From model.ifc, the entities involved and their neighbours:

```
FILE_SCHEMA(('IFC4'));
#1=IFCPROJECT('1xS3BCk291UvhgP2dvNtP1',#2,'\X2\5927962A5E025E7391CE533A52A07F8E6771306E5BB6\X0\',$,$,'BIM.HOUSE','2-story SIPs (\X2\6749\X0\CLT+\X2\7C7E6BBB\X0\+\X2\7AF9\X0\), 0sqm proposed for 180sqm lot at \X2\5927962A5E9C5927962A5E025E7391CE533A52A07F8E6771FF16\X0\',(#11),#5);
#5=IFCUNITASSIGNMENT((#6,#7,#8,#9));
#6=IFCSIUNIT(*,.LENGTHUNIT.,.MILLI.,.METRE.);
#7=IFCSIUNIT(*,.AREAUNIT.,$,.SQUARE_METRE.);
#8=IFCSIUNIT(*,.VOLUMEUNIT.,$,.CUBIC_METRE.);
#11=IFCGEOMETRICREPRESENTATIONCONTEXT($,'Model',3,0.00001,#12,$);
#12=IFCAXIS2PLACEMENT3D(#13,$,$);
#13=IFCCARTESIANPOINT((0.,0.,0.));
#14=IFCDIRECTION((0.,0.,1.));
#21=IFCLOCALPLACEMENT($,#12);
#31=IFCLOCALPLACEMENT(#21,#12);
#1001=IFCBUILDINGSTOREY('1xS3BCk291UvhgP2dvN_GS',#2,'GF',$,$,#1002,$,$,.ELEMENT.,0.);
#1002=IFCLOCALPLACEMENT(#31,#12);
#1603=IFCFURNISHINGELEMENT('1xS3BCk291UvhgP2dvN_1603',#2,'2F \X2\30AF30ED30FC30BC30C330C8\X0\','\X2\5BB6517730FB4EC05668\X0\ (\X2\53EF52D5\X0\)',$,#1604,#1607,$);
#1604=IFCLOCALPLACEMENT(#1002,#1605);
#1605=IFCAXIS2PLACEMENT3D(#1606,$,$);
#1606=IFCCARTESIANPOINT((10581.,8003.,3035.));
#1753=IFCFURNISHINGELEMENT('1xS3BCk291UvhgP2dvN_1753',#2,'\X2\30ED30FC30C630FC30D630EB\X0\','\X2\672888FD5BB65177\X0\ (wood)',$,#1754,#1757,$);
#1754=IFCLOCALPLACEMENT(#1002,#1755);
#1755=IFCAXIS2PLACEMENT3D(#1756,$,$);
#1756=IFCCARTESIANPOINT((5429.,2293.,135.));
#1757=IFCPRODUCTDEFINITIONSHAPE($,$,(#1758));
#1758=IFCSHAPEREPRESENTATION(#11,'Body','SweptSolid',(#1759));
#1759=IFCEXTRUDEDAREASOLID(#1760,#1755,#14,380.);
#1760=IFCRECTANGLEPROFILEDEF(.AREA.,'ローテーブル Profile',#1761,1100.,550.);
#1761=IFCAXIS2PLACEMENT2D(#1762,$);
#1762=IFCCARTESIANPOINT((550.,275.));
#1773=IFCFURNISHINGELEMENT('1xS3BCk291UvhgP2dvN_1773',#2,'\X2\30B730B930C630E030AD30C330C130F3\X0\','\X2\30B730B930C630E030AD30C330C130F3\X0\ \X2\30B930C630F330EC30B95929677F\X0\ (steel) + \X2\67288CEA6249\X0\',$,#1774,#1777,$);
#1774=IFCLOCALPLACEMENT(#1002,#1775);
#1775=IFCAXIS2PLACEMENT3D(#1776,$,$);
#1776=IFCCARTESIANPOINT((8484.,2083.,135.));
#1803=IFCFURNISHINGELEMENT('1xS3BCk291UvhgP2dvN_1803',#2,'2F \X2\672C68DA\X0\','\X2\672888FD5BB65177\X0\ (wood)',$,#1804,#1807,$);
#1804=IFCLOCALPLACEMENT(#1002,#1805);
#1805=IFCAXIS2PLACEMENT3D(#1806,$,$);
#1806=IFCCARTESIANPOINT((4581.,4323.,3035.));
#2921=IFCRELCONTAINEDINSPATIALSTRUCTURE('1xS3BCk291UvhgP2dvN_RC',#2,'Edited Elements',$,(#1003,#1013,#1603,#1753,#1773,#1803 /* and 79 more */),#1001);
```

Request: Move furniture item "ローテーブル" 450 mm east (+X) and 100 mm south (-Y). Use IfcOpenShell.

```python
import ifcopenshell
import ifcopenshell.api.geometry
import ifcopenshell.util.placement

model = ifcopenshell.open("model.ifc")

item = model.by_guid("1xS3BCk291UvhgP2dvN_1753")
matrix = ifcopenshell.util.placement.get_local_placement(item.ObjectPlacement)
matrix[0, 3] += 450.0
matrix[1, 3] -= 100.0
ifcopenshell.api.geometry.edit_object_placement(model, product=item, matrix=matrix, is_si=False)

print(ifcopenshell.util.placement.get_local_placement(item.ObjectPlacement).round(3) + 0.0)

model.write("model_rev.ifc")
```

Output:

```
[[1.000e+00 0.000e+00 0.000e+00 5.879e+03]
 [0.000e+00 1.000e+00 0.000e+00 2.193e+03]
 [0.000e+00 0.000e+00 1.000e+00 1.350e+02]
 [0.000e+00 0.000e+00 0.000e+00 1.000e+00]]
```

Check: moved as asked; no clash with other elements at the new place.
